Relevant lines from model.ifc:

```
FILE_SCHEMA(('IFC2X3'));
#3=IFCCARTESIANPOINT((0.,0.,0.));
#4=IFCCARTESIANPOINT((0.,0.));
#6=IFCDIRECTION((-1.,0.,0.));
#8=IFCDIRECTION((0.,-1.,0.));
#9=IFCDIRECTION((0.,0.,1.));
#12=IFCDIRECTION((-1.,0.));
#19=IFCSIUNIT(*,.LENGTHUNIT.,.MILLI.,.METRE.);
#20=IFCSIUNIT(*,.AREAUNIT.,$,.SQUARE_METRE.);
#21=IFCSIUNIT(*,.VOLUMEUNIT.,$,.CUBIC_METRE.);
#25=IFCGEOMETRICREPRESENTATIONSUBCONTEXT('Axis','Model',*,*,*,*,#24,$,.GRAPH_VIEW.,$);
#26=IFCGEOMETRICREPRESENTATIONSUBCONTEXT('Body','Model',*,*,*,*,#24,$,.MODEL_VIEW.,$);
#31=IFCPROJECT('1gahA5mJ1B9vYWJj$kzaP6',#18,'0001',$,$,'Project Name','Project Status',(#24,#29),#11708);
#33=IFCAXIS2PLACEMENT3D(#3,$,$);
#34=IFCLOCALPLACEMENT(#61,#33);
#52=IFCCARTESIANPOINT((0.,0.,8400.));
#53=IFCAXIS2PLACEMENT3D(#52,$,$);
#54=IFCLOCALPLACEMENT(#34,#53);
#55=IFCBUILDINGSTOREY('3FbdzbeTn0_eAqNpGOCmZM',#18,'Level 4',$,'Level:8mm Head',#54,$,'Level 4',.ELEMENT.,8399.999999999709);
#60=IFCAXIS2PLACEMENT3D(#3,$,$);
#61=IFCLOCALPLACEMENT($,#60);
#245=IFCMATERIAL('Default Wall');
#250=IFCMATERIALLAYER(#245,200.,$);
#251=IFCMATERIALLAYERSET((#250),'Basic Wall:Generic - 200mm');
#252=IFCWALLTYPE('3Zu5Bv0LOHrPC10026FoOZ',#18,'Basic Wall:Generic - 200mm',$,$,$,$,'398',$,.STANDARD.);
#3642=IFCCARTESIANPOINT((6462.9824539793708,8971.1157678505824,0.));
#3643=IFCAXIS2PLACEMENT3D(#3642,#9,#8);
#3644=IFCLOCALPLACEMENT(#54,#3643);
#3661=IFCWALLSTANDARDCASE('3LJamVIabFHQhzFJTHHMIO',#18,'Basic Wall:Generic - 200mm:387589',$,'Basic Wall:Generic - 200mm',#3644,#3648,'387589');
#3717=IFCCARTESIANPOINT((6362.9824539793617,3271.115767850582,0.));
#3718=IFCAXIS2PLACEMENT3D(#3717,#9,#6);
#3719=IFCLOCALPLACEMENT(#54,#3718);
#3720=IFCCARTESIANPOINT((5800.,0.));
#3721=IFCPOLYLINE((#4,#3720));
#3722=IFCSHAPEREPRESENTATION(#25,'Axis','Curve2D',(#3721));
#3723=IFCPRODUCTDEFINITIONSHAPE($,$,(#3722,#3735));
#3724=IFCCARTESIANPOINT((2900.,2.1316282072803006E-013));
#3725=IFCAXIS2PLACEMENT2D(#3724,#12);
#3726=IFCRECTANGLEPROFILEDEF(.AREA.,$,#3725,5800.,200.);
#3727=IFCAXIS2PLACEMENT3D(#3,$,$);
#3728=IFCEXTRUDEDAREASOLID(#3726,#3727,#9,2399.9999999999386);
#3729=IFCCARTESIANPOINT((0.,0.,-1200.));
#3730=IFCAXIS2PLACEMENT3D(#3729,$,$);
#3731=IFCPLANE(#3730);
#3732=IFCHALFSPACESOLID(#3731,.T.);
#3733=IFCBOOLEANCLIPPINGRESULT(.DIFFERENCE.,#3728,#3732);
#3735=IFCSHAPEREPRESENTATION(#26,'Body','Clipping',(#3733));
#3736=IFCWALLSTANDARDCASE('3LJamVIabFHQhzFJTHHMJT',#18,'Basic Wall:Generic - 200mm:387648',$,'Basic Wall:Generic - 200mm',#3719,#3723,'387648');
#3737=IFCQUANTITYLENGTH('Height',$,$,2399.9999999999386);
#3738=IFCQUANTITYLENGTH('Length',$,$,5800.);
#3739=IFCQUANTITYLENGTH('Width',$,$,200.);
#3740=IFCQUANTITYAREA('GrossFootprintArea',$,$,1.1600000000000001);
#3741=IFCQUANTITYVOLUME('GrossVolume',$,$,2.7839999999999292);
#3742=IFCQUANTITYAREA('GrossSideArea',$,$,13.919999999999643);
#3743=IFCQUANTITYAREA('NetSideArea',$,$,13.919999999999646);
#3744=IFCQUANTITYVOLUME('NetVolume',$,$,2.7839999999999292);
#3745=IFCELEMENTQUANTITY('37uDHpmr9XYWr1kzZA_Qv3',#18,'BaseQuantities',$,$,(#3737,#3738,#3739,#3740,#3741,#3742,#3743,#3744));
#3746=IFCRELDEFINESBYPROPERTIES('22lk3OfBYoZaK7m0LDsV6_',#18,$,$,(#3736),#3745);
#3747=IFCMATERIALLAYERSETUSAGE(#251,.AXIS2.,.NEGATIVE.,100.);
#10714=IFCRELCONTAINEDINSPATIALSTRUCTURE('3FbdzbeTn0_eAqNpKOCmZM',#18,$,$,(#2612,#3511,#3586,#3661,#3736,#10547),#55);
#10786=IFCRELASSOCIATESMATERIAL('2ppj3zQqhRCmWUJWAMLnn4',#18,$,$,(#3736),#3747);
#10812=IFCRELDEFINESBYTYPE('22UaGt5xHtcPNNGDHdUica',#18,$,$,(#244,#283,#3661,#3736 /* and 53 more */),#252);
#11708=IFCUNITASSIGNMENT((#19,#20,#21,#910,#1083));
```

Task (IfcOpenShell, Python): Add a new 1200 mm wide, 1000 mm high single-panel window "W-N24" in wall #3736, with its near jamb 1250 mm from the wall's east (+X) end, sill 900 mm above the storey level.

```python
import numpy as np
import ifcopenshell
import ifcopenshell.api.feature
import ifcopenshell.api.geometry
import ifcopenshell.api.pset
import ifcopenshell.api.root
import ifcopenshell.api.spatial
import ifcopenshell.api.type
import ifcopenshell.geom
import ifcopenshell.util.element
import ifcopenshell.util.placement
import ifcopenshell.util.representation
import ifcopenshell.util.shape
import ifcopenshell.util.unit

model = ifcopenshell.open("model.ifc")
unit_scale = ifcopenshell.util.unit.calculate_unit_scale(model)
area_scale = ifcopenshell.util.unit.calculate_unit_scale(model, "AREAUNIT")
volume_scale = ifcopenshell.util.unit.calculate_unit_scale(model, "VOLUMEUNIT")
settings = ifcopenshell.geom.settings()


def volume(element):
    """Net volume in cubic metres, openings subtracted."""
    shape = ifcopenshell.geom.create_shape(settings, element)
    return ifcopenshell.util.shape.get_volume(shape.geometry)


wall = model.by_guid("3LJamVIabFHQhzFJTHHMJT")
storey = ifcopenshell.util.element.get_container(wall, ifc_class="IfcBuildingStorey")
context = ifcopenshell.util.representation.get_context(model, "Model", "Body", "MODEL_VIEW")
before = volume(wall)

width, height, from_end, sill = 1.2, 1, 1.25, 0.9  # metres

# The wall runs along its own X axis, and the end named is its -X end.
wall_shape = ifcopenshell.geom.create_shape(settings, wall)
x, y, z = ifcopenshell.util.shape.get_vertices(wall_shape.geometry).T
start = x.min() + from_end
face, thickness = float(y.min()), float(y.max() - y.min())
wall_matrix = ifcopenshell.util.placement.get_local_placement(wall.ObjectPlacement)
level = ifcopenshell.util.placement.get_local_placement(storey.ObjectPlacement)[2, 3]


def in_wall(x, y):
    """Placement at x, y metres in the wall's axes, at sill height."""
    matrix = wall_matrix.copy()
    matrix[:, 3] = wall_matrix @ np.array([x / unit_scale, y / unit_scale, 0.0, 1.0])
    matrix[2, 3] = level + sill / unit_scale
    return matrix


# Opening: a box that overshoots both wall faces by 50 mm.
opening = ifcopenshell.api.root.create_entity(model, ifc_class="IfcOpeningElement")
box = ifcopenshell.api.geometry.add_wall_representation(
    model, context=context, length=width, height=height, thickness=thickness + 0.1
)
ifcopenshell.api.geometry.assign_representation(model, product=opening, representation=box)
ifcopenshell.api.geometry.edit_object_placement(model, product=opening, matrix=in_wall(start, face - 0.05), is_si=False)
ifcopenshell.api.feature.add_feature(model, feature=opening, element=wall)

window = ifcopenshell.api.root.create_entity(model, ifc_class="IfcWindow", name="W-N24")
window.OverallWidth, window.OverallHeight = width / unit_scale, height / unit_scale
body = ifcopenshell.api.geometry.add_window_representation(
    model,
    context=context,
    overall_width=window.OverallWidth,
    overall_height=window.OverallHeight,
    partition_type="SINGLE_PANEL",
)
ifcopenshell.api.geometry.assign_representation(model, product=window, representation=body)
ifcopenshell.api.spatial.assign_container(model, products=[window], relating_structure=storey)
fills = ifcopenshell.api.feature.add_filling(model, opening=opening, element=window)
fills.OwnerHistory = window.OwnerHistory  # required in IFC2X3

# IFC2X3 keeps the operation on the window style.
style = ifcopenshell.api.root.create_entity(model, ifc_class="IfcWindowStyle", name="W-N24")
style.OperationType, style.ConstructionType = "SINGLE_PANEL", "NOTDEFINED"
style.ParameterTakesPrecedence = style.Sizeable = False
ifcopenshell.api.type.assign_type(model, related_objects=[window], relating_type=style)

# Centre the window in the wall's thickness.
ifcopenshell.api.geometry.edit_object_placement(model, product=window, matrix=in_wall(start, face), is_si=False)
window_shape = ifcopenshell.geom.create_shape(settings, window)
depth = ifcopenshell.util.shape.get_vertices(window_shape.geometry)[:, 1]
offset = face + thickness / 2 - (depth.min() + depth.max()) / 2
ifcopenshell.api.geometry.edit_object_placement(model, product=window, matrix=in_wall(start, offset), is_si=False)

after = volume(wall)

# Update the wall's stored quantities.
qto = model.by_id(ifcopenshell.util.element.get_pset(wall, "BaseQuantities", should_inherit=False)["id"])
ifcopenshell.api.pset.edit_qto(model, qto=qto, properties={
    "NetSideArea": after / thickness / area_scale,
    "NetVolume": after / volume_scale,
})

print(f"wall volume {before:.3f} -> {after:.3f} m3")

model.write("model_updated.ifc")
```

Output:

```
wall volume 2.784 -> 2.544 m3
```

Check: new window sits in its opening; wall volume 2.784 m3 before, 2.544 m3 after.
